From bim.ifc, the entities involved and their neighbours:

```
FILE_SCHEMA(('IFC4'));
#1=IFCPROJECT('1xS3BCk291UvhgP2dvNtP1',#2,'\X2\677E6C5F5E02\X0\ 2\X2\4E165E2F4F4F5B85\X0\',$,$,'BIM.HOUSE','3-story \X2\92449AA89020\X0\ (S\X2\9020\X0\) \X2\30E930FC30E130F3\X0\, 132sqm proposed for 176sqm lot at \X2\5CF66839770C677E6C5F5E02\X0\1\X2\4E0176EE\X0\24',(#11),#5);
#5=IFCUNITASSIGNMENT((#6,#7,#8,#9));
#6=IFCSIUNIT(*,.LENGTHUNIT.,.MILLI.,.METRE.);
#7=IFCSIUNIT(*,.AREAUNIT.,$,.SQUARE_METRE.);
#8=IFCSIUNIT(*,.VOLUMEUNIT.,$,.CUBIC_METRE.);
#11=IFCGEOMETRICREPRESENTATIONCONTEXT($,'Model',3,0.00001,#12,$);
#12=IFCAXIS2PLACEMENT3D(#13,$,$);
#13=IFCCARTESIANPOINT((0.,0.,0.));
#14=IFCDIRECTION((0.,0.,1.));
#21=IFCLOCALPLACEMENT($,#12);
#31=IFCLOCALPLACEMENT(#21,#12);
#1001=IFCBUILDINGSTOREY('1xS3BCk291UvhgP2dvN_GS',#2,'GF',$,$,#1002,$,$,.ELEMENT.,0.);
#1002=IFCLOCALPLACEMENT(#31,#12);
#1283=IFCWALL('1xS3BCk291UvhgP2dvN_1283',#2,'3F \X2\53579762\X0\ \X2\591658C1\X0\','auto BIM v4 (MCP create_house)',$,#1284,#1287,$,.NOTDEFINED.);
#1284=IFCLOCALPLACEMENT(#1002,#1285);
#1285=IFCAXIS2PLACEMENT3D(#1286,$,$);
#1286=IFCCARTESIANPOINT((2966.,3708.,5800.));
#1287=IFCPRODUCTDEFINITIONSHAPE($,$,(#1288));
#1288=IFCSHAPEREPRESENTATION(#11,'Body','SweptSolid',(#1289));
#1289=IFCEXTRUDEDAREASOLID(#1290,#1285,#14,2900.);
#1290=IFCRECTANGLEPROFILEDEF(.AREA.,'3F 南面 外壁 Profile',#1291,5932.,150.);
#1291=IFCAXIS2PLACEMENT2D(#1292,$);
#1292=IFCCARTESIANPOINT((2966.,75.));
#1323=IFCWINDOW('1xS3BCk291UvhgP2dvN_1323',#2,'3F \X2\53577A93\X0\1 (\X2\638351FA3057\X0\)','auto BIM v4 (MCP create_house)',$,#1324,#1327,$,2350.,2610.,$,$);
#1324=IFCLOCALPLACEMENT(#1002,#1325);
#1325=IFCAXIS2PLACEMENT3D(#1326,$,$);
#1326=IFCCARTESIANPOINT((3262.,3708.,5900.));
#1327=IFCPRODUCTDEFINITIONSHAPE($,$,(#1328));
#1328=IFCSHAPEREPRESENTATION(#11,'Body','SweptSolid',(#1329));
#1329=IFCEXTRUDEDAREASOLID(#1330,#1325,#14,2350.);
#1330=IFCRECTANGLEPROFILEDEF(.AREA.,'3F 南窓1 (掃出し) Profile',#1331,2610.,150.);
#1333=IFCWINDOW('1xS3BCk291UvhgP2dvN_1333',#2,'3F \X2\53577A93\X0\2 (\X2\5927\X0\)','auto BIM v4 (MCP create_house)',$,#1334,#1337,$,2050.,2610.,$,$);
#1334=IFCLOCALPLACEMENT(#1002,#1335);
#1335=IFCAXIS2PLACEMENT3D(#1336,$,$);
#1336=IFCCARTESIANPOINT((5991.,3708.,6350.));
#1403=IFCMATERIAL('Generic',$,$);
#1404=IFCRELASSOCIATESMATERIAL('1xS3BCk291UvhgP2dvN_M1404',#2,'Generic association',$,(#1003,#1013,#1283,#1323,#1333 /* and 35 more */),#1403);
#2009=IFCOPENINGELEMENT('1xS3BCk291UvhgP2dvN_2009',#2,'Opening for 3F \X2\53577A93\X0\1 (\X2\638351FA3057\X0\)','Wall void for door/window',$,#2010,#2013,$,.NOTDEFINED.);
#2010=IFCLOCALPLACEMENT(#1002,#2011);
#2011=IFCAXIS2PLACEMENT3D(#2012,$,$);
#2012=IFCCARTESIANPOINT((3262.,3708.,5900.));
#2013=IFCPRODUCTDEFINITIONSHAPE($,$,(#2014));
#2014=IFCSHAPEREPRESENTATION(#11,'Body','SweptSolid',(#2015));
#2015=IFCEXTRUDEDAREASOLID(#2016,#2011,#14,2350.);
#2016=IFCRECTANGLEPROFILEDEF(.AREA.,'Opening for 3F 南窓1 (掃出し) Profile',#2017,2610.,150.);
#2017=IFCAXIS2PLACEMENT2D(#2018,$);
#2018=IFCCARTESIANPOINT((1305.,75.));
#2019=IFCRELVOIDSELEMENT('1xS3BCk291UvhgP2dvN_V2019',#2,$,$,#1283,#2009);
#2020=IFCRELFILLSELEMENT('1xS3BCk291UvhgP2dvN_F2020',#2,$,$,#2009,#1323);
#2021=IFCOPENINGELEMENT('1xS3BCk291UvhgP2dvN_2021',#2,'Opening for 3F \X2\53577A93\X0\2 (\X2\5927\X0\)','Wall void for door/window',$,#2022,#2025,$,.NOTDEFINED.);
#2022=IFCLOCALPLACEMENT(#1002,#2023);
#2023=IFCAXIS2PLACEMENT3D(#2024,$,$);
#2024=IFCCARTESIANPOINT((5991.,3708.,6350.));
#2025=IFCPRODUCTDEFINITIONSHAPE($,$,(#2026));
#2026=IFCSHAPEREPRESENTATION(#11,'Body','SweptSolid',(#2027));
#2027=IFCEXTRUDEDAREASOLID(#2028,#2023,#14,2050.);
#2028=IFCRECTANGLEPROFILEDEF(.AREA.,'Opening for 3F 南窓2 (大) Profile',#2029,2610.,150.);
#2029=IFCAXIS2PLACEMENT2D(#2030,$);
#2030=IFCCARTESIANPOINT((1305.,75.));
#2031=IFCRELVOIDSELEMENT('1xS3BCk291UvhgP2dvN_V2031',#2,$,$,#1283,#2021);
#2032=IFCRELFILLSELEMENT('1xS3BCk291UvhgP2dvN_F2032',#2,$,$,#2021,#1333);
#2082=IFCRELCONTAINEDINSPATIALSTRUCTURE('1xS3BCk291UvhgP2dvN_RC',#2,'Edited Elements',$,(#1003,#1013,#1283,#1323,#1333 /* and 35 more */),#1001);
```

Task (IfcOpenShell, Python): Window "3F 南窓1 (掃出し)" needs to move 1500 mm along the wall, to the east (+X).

```python
import ifcopenshell
import ifcopenshell.api.geometry
import ifcopenshell.util.placement
import ifcopenshell.util.unit

model = ifcopenshell.open("bim.ifc")
unit_scale = ifcopenshell.util.unit.calculate_unit_scale(model)

window = model.by_id(1323)
opening = window.FillsVoids[0].RelatingOpeningElement
wall = opening.VoidsElements[0].RelatingBuildingElement

wall_matrix = ifcopenshell.util.placement.get_local_placement(wall.ObjectPlacement)
shift = wall_matrix[:3, 0] * 1.5 / unit_scale
before = ifcopenshell.util.placement.get_local_placement(window.ObjectPlacement)[:3, 3].copy()

# The window is not placed relative to its opening, so move both.
for product in (opening, window):
    matrix = ifcopenshell.util.placement.get_local_placement(product.ObjectPlacement)
    matrix[:3, 3] += shift
    ifcopenshell.api.geometry.edit_object_placement(model, product=product, matrix=matrix, is_si=False)

after = ifcopenshell.util.placement.get_local_placement(window.ObjectPlacement)[:3, 3]
print("window moved by", (after - before).round(3) + 0.0)

model.write("bim-out.ifc")
```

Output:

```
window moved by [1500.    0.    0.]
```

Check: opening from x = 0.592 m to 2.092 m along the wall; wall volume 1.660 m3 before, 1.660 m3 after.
